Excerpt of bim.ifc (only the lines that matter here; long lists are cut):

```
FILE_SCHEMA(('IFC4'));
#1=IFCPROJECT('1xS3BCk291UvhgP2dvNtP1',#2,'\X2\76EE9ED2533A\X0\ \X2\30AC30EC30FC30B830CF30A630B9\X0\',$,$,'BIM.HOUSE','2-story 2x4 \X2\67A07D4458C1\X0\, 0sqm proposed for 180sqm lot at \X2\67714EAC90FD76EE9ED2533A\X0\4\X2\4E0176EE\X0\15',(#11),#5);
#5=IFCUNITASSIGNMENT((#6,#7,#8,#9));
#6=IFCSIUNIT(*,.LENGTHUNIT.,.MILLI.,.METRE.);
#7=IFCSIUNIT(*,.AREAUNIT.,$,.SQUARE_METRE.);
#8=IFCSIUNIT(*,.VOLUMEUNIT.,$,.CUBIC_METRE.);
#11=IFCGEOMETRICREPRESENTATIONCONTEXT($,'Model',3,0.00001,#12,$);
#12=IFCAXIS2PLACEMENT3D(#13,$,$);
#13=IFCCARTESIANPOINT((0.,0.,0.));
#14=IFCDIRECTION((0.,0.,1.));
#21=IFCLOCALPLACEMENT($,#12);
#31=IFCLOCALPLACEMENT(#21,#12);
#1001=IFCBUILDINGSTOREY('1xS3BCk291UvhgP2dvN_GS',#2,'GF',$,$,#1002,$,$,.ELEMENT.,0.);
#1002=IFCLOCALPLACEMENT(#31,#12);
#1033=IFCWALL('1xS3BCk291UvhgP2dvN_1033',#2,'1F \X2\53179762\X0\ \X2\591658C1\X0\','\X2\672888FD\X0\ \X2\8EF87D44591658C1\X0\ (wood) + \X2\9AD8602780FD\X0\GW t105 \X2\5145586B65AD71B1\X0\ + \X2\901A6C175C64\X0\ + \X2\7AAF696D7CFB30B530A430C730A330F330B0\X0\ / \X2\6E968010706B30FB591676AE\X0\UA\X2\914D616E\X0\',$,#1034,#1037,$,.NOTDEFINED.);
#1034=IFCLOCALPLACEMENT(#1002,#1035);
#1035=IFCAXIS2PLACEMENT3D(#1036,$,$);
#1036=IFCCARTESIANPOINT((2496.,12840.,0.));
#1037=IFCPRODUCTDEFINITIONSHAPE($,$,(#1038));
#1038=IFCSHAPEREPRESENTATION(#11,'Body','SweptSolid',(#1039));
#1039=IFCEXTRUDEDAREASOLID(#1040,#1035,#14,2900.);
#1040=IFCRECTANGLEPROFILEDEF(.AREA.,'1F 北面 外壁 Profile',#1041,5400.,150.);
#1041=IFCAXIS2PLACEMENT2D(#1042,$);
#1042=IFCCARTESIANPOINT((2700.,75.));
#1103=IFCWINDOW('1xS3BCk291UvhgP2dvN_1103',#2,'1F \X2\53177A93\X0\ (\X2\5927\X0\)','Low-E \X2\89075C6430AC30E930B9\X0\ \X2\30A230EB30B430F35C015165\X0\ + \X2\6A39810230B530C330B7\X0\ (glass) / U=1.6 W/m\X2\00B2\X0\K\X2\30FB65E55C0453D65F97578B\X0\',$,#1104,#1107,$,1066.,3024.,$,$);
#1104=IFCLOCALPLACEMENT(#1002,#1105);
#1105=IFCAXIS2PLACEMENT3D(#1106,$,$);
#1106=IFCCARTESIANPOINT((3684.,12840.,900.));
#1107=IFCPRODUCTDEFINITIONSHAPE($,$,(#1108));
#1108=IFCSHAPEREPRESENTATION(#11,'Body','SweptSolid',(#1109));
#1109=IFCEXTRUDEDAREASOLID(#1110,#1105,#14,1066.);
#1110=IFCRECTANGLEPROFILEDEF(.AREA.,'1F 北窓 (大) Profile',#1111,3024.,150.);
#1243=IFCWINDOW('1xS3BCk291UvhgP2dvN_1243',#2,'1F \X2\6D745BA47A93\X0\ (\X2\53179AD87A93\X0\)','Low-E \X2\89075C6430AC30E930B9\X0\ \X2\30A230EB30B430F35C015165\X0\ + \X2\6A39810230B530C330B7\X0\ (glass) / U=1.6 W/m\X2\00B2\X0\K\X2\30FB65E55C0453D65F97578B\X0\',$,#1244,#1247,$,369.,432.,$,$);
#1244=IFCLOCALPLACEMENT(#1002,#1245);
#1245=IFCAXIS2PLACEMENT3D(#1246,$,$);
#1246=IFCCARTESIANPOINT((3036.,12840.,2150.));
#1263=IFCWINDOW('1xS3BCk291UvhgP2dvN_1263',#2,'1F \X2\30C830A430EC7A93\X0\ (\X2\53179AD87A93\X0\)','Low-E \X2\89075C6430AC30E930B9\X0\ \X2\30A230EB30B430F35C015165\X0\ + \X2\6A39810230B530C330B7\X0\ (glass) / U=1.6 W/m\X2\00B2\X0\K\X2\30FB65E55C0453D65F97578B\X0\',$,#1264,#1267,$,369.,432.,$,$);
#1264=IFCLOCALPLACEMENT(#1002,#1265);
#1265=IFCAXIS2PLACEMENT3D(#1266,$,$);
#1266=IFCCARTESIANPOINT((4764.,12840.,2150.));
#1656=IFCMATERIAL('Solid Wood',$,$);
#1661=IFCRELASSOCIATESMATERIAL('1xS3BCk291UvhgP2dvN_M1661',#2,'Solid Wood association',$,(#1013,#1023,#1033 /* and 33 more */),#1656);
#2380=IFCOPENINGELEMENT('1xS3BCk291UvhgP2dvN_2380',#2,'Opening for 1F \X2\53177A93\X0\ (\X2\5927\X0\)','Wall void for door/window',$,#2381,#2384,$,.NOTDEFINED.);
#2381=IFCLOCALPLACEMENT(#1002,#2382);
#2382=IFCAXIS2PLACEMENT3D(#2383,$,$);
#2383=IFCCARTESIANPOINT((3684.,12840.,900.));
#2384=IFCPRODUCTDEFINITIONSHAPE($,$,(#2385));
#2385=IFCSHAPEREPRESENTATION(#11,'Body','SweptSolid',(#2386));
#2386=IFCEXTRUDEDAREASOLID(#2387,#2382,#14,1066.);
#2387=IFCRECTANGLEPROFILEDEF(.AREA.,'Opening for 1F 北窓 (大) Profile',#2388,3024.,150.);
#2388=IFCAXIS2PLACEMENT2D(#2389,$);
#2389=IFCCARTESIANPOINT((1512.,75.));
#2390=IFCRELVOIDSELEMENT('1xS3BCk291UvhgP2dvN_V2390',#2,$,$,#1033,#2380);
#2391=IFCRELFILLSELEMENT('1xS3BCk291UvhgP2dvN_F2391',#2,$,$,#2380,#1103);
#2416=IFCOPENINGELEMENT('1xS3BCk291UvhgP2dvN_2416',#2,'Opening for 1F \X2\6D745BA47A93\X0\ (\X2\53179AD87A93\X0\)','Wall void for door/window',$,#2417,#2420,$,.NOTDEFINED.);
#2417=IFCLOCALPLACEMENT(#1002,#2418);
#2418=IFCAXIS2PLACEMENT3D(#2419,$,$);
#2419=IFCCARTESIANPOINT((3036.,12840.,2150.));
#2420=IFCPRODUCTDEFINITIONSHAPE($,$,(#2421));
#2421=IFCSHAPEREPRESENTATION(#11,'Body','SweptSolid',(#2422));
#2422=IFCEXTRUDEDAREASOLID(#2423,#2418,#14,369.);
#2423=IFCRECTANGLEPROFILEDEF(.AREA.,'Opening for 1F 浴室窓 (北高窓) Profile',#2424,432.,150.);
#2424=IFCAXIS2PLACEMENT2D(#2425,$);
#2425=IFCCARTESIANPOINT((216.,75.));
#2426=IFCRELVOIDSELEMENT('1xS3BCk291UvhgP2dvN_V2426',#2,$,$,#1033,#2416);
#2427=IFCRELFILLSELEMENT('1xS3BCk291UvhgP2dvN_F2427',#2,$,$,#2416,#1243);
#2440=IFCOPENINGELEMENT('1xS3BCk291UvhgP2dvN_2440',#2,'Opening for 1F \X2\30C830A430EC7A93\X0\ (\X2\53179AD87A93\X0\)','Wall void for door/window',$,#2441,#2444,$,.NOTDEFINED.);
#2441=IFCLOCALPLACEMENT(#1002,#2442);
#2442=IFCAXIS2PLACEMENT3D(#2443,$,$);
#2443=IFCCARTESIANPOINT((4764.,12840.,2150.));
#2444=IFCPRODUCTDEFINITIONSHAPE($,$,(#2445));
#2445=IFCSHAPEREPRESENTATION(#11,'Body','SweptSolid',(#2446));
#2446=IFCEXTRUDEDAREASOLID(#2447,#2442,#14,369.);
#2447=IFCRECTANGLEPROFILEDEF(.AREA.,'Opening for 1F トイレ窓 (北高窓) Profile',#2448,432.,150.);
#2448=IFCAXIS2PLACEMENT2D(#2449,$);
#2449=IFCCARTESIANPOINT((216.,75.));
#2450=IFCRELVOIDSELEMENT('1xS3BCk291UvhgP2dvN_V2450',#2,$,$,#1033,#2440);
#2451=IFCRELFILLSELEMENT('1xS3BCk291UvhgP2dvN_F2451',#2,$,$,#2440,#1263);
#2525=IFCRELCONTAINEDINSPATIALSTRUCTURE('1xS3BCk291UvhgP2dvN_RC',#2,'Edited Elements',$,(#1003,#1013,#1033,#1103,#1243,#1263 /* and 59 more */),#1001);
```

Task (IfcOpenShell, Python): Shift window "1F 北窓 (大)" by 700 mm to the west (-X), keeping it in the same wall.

```python
import ifcopenshell
import ifcopenshell.api.geometry
import ifcopenshell.util.placement

model = ifcopenshell.open("bim.ifc")

window = model.by_guid("1xS3BCk291UvhgP2dvN_1103")
opening = window.FillsVoids[0].RelatingOpeningElement
wall = opening.VoidsElements[0].RelatingBuildingElement

wall_matrix = ifcopenshell.util.placement.get_local_placement(wall.ObjectPlacement)
shift = wall_matrix[:3, 0] * -700.0
before = ifcopenshell.util.placement.get_local_placement(window.ObjectPlacement)[:3, 3].copy()

# The window is not placed relative to its opening, so move both.
for product in (opening, window):
    matrix = ifcopenshell.util.placement.get_local_placement(product.ObjectPlacement)
    matrix[:3, 3] += shift
    ifcopenshell.api.geometry.edit_object_placement(model, product=product, matrix=matrix, is_si=False)

after = ifcopenshell.util.placement.get_local_placement(window.ObjectPlacement)[:3, 3]
print("window moved by", (after - before).round(3) + 0.0)

model.write("bim_v2.ifc")
```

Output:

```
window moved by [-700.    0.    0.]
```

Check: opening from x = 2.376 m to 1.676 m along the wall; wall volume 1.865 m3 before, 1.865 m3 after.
